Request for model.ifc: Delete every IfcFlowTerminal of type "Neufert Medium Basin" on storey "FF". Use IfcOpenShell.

First a look at what the model holds.

```python
import ifcopenshell
import ifcopenshell.util.element

model = ifcopenshell.open("model.ifc")
print(model.schema)
storey = next(s for s in model.by_type("IfcBuildingStorey") if s.Name == "FF")
terminals = [e for e in ifcopenshell.util.element.get_decomposition(storey) if e.is_a("IfcFlowTerminal")]
seen = {}
for e in terminals:
    element_type = ifcopenshell.util.element.get_type(e)
    name = element_type.Name if element_type not in (None, e) else None
    seen[name] = seen.get(name, 0) + 1
for name, count in sorted(seen.items(), key=str):
    print(count, "x", name)
```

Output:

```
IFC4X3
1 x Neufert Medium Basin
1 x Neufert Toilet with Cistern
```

```python
import ifcopenshell
import ifcopenshell.api.root
import ifcopenshell.util.element

model = ifcopenshell.open("model.ifc")

storey = next(s for s in model.by_type("IfcBuildingStorey") if s.Name == "FF")
terminals = [e for e in ifcopenshell.util.element.get_decomposition(storey) if e.is_a("IfcFlowTerminal")]
targets = [e for e in terminals if (t := ifcopenshell.util.element.get_type(e)) not in (None, e) and t.Name == "Neufert Medium Basin"]

for e in targets:
    ifcopenshell.api.root.remove_product(model, product=e)
print(len(targets), "removed")

model.write("model-out.ifc")
```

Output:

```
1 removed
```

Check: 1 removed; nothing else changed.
